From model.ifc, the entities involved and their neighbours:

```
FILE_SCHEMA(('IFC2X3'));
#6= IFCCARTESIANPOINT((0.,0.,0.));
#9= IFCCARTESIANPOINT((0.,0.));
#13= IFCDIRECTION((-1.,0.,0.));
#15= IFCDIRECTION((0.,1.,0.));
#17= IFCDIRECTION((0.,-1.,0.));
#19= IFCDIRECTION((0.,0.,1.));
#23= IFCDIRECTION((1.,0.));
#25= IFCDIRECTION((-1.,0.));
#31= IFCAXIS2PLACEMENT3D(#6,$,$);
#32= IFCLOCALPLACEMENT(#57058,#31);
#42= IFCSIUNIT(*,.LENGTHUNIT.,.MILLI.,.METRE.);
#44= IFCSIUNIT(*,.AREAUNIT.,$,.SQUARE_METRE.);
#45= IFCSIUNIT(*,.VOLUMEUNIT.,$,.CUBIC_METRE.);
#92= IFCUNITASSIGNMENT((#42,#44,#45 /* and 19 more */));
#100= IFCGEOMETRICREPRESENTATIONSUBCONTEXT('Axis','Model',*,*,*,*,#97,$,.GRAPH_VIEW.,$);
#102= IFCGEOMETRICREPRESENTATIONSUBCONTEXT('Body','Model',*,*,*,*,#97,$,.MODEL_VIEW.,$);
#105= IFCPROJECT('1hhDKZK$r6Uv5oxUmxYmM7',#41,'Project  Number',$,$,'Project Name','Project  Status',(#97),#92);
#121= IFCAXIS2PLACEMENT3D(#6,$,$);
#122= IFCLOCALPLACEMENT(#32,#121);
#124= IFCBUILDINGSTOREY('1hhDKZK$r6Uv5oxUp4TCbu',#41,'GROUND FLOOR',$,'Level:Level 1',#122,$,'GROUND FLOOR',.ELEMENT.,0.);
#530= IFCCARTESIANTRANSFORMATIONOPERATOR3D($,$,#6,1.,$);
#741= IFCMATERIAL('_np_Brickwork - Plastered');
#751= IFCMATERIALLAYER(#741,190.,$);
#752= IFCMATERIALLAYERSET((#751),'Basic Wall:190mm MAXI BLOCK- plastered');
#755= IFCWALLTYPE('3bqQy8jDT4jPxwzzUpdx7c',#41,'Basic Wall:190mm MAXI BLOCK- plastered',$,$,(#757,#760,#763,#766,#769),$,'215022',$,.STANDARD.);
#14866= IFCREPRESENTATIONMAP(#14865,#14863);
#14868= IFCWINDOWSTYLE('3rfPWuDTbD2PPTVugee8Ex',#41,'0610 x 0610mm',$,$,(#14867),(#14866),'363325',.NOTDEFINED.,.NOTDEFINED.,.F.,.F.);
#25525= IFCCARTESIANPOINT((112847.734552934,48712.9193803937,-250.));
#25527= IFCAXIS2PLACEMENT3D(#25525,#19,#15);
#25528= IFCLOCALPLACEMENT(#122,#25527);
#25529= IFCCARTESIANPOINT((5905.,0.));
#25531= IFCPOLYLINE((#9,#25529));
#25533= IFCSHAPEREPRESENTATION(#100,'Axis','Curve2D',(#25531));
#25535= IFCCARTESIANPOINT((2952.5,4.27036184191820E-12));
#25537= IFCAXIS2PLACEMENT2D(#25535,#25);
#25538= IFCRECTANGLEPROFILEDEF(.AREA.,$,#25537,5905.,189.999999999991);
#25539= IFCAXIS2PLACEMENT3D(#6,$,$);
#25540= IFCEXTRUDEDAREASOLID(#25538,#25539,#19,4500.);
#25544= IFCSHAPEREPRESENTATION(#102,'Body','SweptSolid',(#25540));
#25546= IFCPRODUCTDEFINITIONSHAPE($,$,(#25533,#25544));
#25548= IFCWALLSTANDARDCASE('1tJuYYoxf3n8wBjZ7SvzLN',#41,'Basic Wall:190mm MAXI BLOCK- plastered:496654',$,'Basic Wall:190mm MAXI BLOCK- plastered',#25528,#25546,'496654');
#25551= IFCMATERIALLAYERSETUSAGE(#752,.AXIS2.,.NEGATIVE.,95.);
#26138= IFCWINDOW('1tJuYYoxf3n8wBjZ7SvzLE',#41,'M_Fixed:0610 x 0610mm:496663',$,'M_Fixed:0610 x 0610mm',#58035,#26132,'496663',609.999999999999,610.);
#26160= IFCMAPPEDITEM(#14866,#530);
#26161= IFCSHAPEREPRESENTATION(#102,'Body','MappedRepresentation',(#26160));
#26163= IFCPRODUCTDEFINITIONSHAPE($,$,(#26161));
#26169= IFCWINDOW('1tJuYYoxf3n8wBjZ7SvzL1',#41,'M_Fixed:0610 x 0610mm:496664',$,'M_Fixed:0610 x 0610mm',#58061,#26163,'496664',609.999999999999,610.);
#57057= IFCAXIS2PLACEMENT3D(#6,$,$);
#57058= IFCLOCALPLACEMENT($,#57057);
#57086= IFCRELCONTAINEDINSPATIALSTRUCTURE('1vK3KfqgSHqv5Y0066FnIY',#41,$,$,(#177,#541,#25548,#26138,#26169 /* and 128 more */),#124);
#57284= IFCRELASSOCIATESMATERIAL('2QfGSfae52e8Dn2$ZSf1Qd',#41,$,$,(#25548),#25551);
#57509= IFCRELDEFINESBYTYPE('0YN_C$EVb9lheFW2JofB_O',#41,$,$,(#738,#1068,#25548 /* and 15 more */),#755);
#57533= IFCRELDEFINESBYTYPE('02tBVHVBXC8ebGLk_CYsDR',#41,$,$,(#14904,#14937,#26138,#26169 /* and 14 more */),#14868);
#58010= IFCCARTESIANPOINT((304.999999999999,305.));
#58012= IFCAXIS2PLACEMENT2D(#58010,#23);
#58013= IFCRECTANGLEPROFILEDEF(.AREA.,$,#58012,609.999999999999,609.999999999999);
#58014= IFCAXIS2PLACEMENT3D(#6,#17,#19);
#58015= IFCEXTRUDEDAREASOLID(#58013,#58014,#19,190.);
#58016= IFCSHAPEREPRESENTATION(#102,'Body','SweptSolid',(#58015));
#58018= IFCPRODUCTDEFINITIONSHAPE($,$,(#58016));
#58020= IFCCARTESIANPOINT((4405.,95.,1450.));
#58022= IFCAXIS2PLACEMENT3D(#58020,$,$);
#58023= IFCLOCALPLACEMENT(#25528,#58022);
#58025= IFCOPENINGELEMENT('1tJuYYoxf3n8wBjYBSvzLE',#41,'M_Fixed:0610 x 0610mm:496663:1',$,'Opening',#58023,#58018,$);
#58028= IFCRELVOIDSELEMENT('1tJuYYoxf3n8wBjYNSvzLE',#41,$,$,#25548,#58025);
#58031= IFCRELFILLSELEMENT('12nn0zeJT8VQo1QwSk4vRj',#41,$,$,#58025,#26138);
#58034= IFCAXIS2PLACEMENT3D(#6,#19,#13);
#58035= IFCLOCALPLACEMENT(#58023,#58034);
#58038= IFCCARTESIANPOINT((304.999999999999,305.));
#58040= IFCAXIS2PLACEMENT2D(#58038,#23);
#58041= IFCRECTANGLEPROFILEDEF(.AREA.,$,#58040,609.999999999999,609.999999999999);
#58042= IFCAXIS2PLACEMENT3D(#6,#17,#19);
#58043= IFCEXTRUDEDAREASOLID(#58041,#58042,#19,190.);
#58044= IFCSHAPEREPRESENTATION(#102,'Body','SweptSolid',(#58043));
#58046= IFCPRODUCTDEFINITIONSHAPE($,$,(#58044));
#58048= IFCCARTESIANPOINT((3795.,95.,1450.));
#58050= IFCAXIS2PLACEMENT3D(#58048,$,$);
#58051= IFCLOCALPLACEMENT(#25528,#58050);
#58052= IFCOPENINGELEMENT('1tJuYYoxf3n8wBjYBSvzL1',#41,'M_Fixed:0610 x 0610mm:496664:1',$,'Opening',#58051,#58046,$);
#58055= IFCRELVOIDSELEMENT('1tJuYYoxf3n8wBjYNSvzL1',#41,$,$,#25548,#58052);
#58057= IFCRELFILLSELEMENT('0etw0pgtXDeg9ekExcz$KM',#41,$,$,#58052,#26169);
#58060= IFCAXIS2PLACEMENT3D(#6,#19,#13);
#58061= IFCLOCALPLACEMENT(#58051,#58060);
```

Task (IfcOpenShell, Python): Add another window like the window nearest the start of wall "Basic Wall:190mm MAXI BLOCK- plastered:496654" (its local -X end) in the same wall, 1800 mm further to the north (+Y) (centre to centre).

```python
import ifcopenshell
import ifcopenshell.api.feature
import ifcopenshell.api.geometry
import ifcopenshell.api.root
import ifcopenshell.geom
import ifcopenshell.util.element
import ifcopenshell.util.placement
import ifcopenshell.util.shape

model = ifcopenshell.open("model.ifc")
settings = ifcopenshell.geom.settings()


def volume(element):
    """Net volume in cubic metres, openings subtracted."""
    shape = ifcopenshell.geom.create_shape(settings, element)
    return ifcopenshell.util.shape.get_volume(shape.geometry)


def reuse_history(source, copy):
    """copy_class also copies each property set's owner history, people and application; keep the originals."""
    for rel in copy.IsDefinedBy:
        if rel.is_a("IfcRelDefinesByProperties") and (history := rel.RelatingPropertyDefinition.OwnerHistory):
            rel.RelatingPropertyDefinition.OwnerHistory = source.OwnerHistory
            ifcopenshell.util.element.remove_deep2(model, history)


window = model.by_id(26169)
opening = window.FillsVoids[0].RelatingOpeningElement
wall = opening.VoidsElements[0].RelatingBuildingElement
before = volume(wall)
shift = ifcopenshell.util.placement.get_local_placement(wall.ObjectPlacement)[:3, 0] * 1800.0

# copy_class copies the void relationship, type, container and properties, but no geometry.
new_opening = ifcopenshell.api.root.copy_class(model, product=opening)
new_opening.Representation = ifcopenshell.util.element.copy_deep(
    model, opening.Representation, exclude=["IfcGeometricRepresentationContext", "IfcRepresentationMap"]
)
new_opening.Name = "M_Fixed:0610 x 0610mm"
new_window = ifcopenshell.api.root.copy_class(model, product=window)
new_window.Representation = ifcopenshell.util.element.copy_deep(
    model, window.Representation, exclude=["IfcGeometricRepresentationContext", "IfcRepresentationMap"]
)
new_window.Name = "M_Fixed:0610 x 0610mm"
new_window.Tag = None
reuse_history(window, new_window)
fills = ifcopenshell.api.feature.add_filling(model, opening=new_opening, element=new_window)
fills.OwnerHistory = new_window.OwnerHistory  # required in IFC2X3

for old, new in ((opening, new_opening), (window, new_window)):
    matrix = ifcopenshell.util.placement.get_local_placement(old.ObjectPlacement)
    matrix[:3, 3] += shift
    ifcopenshell.api.geometry.edit_object_placement(model, product=new, matrix=matrix, is_si=False)

after = volume(wall)

print(f"wall volume {before:.3f} -> {after:.3f} m3")

model.write("model-out.ifc")
```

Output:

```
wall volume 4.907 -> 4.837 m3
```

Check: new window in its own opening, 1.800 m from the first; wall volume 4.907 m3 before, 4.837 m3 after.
